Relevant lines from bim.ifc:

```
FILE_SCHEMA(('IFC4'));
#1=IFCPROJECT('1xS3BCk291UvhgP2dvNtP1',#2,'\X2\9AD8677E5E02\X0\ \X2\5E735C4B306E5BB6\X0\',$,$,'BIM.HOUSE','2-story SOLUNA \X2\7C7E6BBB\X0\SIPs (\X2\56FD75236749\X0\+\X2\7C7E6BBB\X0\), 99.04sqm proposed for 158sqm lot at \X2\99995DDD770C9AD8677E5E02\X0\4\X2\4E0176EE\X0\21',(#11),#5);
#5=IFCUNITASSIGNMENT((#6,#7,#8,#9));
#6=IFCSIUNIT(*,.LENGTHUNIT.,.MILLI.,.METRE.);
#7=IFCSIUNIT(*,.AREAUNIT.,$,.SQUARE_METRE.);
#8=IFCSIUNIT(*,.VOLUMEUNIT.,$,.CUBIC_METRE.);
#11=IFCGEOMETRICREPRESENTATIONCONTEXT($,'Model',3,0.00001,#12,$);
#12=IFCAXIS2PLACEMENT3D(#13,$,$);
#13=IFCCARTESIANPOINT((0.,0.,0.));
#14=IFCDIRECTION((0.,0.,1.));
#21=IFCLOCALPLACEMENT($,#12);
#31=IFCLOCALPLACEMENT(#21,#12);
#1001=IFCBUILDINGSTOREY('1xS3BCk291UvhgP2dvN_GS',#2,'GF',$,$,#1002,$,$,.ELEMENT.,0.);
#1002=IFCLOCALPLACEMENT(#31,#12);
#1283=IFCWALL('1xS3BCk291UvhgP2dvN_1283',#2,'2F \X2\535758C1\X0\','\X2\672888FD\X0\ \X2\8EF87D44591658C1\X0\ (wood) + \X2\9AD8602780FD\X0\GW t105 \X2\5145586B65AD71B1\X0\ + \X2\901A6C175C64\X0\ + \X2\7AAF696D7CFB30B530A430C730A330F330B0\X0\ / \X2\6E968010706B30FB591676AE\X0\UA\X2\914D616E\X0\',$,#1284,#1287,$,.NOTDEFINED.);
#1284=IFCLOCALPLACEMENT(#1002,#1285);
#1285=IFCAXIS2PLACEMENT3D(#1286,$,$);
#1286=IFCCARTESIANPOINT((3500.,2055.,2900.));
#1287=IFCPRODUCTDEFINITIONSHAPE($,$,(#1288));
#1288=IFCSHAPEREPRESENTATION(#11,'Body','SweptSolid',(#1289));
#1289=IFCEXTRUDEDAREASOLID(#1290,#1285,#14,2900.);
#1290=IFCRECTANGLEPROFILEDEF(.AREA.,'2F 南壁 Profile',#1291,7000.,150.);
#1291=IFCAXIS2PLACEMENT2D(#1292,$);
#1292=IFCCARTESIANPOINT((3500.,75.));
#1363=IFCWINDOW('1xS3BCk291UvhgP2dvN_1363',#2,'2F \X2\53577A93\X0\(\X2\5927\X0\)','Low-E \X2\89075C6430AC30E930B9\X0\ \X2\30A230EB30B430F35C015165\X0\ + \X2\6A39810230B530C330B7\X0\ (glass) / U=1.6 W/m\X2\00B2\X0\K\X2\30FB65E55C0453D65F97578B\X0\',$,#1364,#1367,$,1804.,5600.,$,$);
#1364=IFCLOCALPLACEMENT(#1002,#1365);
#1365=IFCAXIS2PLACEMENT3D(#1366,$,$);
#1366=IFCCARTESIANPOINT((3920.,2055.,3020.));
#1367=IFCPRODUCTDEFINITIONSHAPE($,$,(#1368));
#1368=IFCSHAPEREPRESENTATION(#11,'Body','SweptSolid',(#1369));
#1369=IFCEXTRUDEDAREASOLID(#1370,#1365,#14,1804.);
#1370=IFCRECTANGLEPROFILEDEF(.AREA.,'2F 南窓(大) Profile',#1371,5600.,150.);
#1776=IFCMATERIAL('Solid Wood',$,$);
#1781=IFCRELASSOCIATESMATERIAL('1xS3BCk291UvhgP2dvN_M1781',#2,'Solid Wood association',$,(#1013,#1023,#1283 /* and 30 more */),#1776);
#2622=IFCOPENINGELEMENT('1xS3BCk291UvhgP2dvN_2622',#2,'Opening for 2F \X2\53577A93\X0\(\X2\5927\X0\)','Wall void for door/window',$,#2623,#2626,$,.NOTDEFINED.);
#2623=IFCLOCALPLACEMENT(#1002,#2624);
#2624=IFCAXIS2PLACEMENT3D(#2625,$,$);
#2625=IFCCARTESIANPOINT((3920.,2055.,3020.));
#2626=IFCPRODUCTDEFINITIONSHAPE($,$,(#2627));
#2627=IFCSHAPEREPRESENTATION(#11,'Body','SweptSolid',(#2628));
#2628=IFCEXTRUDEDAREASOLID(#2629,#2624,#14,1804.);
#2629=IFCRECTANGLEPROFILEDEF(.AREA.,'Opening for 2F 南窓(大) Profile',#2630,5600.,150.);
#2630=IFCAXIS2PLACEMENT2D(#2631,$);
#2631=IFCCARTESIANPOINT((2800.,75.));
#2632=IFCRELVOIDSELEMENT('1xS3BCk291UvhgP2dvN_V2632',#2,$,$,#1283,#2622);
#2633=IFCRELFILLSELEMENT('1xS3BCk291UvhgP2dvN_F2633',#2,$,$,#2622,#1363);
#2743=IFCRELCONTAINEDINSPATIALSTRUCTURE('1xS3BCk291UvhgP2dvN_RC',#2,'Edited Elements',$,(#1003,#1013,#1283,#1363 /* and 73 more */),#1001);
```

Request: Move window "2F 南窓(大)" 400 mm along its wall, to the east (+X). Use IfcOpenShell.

```python
import ifcopenshell
import ifcopenshell.api.geometry
import ifcopenshell.util.placement

model = ifcopenshell.open("bim.ifc")

window = model.by_guid("1xS3BCk291UvhgP2dvN_1363")
opening = window.FillsVoids[0].RelatingOpeningElement
wall = opening.VoidsElements[0].RelatingBuildingElement

wall_matrix = ifcopenshell.util.placement.get_local_placement(wall.ObjectPlacement)
shift = wall_matrix[:3, 0] * 400.0
before = ifcopenshell.util.placement.get_local_placement(window.ObjectPlacement)[:3, 3].copy()

# The window is not placed relative to its opening, so move both.
for product in (opening, window):
    matrix = ifcopenshell.util.placement.get_local_placement(product.ObjectPlacement)
    matrix[:3, 3] += shift
    ifcopenshell.api.geometry.edit_object_placement(model, product=product, matrix=matrix, is_si=False)

after = ifcopenshell.util.placement.get_local_placement(window.ObjectPlacement)[:3, 3]
print("window moved by", (after - before).round(3) + 0.0)

model.write("bim_v2.ifc")
```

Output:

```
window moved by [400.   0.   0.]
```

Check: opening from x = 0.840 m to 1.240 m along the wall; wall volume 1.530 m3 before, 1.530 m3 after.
